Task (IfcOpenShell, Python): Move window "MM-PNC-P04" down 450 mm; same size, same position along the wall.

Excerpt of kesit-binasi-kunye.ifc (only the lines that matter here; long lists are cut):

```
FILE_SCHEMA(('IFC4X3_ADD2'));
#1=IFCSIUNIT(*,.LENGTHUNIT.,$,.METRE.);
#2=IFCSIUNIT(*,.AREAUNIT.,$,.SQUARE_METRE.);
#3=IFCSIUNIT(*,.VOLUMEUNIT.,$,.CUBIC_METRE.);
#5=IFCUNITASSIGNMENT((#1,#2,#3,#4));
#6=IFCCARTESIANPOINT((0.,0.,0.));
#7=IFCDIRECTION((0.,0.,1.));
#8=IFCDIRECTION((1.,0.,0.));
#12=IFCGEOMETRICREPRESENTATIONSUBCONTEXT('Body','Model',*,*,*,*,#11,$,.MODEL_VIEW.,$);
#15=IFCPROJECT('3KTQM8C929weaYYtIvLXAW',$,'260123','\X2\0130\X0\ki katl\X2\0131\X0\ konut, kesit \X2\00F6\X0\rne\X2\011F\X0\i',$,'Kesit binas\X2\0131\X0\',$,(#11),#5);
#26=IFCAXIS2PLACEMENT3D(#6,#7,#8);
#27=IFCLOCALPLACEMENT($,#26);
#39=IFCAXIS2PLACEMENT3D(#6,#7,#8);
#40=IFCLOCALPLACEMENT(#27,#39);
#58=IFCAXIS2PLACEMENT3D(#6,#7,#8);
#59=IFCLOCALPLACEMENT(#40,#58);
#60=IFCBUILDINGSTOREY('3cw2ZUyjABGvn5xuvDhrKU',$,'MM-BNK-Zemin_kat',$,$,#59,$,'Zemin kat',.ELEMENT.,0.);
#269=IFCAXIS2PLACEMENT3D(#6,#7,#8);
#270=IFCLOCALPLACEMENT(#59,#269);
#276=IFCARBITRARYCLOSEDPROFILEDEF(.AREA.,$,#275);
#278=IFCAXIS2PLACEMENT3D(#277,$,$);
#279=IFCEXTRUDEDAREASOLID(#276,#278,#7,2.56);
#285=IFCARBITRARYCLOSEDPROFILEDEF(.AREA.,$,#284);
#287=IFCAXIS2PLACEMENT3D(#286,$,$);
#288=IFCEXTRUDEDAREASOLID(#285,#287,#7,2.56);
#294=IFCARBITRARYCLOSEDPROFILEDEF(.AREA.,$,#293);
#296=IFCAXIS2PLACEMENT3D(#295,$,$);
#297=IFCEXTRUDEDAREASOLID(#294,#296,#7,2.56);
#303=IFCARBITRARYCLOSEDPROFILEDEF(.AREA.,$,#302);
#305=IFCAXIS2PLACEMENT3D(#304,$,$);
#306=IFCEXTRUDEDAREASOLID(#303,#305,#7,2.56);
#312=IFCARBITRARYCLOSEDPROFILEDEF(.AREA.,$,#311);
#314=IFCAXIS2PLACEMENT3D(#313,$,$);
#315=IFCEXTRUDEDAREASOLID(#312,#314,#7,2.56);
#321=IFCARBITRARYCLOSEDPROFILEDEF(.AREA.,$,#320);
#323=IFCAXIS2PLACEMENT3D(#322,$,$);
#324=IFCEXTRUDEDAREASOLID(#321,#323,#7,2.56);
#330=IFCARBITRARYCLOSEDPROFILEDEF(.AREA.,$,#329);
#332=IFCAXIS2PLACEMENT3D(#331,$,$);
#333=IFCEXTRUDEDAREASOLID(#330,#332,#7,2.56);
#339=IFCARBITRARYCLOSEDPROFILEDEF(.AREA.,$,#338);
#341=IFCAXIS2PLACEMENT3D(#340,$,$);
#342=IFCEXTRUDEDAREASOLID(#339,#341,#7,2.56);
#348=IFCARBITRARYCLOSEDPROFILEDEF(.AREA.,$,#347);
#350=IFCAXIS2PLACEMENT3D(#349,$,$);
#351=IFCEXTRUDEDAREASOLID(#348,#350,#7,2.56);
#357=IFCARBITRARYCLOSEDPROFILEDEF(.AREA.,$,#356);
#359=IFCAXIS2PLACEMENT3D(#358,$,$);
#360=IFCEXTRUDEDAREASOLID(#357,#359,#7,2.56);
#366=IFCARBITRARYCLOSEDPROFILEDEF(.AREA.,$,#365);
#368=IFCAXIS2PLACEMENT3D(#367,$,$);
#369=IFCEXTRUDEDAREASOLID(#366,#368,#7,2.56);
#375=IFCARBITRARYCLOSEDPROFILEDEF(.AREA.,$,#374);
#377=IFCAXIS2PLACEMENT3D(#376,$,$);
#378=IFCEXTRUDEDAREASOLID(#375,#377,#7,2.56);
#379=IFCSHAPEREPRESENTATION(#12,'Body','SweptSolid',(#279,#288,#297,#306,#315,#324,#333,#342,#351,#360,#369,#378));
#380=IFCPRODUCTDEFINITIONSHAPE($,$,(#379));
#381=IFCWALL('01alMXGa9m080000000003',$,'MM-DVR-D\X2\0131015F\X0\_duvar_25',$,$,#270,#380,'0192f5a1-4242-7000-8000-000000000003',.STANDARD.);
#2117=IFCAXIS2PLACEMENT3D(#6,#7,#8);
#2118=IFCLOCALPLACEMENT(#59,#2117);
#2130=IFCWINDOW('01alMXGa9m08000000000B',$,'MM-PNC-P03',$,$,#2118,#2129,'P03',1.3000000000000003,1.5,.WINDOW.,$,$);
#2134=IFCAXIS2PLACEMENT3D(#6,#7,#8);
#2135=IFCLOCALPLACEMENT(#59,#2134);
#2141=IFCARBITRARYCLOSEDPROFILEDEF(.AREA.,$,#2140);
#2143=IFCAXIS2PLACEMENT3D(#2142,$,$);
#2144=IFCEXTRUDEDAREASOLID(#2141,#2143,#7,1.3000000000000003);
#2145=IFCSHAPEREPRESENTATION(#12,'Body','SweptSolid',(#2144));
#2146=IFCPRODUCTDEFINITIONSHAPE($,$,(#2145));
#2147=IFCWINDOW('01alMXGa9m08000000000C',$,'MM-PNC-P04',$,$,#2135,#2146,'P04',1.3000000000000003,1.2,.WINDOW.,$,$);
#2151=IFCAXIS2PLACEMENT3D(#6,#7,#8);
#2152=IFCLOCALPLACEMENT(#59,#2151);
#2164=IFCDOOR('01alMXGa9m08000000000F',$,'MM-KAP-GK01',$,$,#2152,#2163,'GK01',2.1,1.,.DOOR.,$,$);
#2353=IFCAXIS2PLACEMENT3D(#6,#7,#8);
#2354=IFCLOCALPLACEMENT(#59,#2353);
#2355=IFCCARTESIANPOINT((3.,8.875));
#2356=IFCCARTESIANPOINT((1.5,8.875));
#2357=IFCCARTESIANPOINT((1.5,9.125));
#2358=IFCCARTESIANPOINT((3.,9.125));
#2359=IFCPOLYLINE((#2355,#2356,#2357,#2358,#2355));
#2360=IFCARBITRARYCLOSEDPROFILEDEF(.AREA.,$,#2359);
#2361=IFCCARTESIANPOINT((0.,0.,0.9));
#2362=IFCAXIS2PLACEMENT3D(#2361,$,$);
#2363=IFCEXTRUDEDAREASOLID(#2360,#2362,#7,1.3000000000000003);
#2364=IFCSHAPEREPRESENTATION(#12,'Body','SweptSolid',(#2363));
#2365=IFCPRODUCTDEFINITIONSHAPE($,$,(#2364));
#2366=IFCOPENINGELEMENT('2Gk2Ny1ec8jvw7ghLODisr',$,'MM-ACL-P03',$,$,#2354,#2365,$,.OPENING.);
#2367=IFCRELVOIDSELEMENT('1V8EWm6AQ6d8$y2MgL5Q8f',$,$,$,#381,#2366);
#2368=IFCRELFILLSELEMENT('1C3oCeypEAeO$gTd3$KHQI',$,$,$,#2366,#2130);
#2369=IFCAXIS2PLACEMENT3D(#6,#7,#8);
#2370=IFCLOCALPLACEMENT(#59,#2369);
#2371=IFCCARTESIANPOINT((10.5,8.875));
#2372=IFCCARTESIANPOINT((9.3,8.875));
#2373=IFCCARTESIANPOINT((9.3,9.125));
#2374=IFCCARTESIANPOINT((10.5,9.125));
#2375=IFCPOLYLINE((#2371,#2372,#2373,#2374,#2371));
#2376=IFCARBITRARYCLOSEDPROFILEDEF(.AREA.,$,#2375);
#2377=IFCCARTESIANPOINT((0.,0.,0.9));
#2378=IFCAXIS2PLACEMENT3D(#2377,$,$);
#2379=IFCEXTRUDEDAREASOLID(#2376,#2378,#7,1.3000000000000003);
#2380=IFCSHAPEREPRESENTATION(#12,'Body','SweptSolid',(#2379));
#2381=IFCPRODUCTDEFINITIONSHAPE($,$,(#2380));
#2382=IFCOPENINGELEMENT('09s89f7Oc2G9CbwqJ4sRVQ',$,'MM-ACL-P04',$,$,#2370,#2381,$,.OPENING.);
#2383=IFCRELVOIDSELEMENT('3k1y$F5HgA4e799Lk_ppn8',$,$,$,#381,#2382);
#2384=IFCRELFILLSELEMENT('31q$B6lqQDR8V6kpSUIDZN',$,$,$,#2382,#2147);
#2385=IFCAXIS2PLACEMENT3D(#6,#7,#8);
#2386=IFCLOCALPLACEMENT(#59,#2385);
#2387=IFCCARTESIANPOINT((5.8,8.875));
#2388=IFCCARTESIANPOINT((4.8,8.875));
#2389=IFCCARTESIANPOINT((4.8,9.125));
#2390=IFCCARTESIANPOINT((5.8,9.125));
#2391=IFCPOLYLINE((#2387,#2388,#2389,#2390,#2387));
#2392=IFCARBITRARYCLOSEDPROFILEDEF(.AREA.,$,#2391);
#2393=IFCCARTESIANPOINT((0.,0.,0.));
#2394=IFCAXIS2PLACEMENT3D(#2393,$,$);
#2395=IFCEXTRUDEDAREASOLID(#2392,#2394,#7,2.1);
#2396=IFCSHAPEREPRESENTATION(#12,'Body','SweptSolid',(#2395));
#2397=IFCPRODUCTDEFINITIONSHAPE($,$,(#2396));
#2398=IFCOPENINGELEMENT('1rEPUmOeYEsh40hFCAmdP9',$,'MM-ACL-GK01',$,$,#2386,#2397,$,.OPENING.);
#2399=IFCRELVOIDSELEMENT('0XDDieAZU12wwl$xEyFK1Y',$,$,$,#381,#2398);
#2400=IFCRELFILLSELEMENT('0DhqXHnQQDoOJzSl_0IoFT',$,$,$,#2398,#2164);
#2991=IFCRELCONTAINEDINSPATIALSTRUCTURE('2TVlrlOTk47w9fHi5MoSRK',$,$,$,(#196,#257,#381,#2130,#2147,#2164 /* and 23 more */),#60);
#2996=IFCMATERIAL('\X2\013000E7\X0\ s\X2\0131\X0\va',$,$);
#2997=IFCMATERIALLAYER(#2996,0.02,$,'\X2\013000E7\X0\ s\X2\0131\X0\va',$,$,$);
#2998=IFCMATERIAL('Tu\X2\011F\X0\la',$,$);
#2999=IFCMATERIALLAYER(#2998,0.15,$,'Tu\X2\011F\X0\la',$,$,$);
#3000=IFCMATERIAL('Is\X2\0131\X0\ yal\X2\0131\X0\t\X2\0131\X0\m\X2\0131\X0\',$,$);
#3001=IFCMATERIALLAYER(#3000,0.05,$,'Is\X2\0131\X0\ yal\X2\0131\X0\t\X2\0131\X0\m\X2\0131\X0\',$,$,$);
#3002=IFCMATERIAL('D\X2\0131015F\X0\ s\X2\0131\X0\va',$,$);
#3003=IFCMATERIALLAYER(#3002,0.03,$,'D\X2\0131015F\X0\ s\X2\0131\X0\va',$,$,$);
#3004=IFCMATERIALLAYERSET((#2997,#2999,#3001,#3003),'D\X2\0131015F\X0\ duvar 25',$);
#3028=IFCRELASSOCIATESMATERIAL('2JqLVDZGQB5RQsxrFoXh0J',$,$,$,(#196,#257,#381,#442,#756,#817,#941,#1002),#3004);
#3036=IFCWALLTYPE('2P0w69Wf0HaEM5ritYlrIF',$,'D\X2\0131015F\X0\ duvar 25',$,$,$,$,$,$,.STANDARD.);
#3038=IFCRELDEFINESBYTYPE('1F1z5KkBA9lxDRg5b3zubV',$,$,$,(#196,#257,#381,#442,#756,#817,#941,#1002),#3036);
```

```python
import numpy as np
import ifcopenshell
import ifcopenshell.api.geometry
import ifcopenshell.util.placement
import ifcopenshell.util.unit

model = ifcopenshell.open("kesit-binasi-kunye.ifc")
unit_scale = ifcopenshell.util.unit.calculate_unit_scale(model)

window = model.by_guid("01alMXGa9m08000000000C")
opening = window.FillsVoids[0].RelatingOpeningElement
dz = -0.45 / unit_scale

shift = np.array([0.0, 0.0, dz])
# The window is not placed relative to its opening, so move both.
for product in (opening, window):
    matrix = ifcopenshell.util.placement.get_local_placement(product.ObjectPlacement)
    matrix[:3, 3] += shift
    ifcopenshell.api.geometry.edit_object_placement(model, product=product, matrix=matrix, is_si=False)

print(f"moved by {dz * unit_scale:+.3f} m")

model.write("kesit-binasi-kunye_v2.ifc")
```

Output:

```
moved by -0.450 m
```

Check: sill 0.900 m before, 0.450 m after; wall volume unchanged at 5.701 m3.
